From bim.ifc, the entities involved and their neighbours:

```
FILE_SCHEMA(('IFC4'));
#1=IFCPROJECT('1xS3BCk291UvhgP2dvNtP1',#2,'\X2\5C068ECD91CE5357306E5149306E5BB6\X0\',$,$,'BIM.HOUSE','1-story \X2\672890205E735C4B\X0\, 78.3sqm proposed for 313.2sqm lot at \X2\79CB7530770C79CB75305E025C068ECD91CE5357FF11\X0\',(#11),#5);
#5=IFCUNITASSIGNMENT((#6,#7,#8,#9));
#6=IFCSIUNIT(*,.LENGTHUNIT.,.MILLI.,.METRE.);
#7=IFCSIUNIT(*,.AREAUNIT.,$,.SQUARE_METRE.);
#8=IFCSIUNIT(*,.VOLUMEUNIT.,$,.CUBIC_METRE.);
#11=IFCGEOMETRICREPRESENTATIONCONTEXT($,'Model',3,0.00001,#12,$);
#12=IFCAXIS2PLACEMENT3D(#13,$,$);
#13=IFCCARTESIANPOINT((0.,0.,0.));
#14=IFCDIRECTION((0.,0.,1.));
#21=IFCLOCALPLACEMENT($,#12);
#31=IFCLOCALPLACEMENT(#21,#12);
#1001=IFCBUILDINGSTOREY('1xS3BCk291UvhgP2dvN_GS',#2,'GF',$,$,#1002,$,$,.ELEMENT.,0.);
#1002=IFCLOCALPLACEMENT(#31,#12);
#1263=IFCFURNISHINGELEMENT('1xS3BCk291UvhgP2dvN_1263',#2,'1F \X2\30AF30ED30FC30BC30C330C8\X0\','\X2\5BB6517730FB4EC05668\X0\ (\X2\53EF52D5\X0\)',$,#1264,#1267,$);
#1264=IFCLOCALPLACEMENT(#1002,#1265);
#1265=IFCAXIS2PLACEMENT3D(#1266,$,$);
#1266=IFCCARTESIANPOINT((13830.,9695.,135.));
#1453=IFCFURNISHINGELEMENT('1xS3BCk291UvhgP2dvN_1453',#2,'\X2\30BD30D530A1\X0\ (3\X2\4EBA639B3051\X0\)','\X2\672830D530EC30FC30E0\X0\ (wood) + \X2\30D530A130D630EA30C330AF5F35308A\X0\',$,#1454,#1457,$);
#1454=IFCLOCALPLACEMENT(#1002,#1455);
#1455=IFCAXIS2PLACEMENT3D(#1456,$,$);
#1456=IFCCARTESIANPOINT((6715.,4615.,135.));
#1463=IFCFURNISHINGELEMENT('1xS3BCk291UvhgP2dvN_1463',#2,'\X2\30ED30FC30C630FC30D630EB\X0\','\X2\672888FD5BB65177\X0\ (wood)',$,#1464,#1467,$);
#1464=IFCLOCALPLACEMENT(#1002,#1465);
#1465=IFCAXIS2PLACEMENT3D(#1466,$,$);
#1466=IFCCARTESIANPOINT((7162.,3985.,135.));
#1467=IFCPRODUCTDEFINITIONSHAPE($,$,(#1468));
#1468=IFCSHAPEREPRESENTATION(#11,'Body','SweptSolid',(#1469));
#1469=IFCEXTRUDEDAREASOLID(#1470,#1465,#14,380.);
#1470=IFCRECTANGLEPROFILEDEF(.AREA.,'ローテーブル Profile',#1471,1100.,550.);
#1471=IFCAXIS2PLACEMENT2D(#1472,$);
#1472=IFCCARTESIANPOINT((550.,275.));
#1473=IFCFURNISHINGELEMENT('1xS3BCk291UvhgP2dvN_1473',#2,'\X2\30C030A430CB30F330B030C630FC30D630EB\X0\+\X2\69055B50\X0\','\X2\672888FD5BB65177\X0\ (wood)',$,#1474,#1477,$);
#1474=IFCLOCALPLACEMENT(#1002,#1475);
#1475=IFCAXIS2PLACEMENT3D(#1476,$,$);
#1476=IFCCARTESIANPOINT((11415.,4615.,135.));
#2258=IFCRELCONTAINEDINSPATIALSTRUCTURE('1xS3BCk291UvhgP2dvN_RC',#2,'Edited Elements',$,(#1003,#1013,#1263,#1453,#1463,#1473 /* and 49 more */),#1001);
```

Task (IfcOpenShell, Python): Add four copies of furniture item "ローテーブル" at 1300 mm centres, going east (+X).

```python
import numpy as np
import ifcopenshell
import ifcopenshell.api.geometry
import ifcopenshell.api.root
import ifcopenshell.util.element
import ifcopenshell.util.placement

model = ifcopenshell.open("bim.ifc")


def reuse_history(source, copy):
    """copy_class also copies each property set's owner history, people and application; keep the originals."""
    for rel in copy.IsDefinedBy:
        if rel.is_a("IfcRelDefinesByProperties") and (history := rel.RelatingPropertyDefinition.OwnerHistory):
            rel.RelatingPropertyDefinition.OwnerHistory = source.OwnerHistory
            ifcopenshell.util.element.remove_deep2(model, history)


source = model.by_guid("1xS3BCk291UvhgP2dvN_1463")
base = ifcopenshell.util.placement.get_local_placement(source.ObjectPlacement)
step = np.array([1.0, 0.0, 0.0]) * 1300.0

for i in range(1, 5):
    copy = ifcopenshell.api.root.copy_class(model, product=source)
    copy.Representation = ifcopenshell.util.element.copy_deep(
        model, source.Representation, exclude=["IfcGeometricRepresentationContext", "IfcRepresentationMap"]
    )
    reuse_history(source, copy)
    matrix = base.copy()
    matrix[:3, 3] += i * step
    print("added at", matrix[:3, 3].round(3) + 0.0)
    ifcopenshell.api.geometry.edit_object_placement(model, product=copy, matrix=matrix, is_si=False)

model.write("bim-out.ifc")
```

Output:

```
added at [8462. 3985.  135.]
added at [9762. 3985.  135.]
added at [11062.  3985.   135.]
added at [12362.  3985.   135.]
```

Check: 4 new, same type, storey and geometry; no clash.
